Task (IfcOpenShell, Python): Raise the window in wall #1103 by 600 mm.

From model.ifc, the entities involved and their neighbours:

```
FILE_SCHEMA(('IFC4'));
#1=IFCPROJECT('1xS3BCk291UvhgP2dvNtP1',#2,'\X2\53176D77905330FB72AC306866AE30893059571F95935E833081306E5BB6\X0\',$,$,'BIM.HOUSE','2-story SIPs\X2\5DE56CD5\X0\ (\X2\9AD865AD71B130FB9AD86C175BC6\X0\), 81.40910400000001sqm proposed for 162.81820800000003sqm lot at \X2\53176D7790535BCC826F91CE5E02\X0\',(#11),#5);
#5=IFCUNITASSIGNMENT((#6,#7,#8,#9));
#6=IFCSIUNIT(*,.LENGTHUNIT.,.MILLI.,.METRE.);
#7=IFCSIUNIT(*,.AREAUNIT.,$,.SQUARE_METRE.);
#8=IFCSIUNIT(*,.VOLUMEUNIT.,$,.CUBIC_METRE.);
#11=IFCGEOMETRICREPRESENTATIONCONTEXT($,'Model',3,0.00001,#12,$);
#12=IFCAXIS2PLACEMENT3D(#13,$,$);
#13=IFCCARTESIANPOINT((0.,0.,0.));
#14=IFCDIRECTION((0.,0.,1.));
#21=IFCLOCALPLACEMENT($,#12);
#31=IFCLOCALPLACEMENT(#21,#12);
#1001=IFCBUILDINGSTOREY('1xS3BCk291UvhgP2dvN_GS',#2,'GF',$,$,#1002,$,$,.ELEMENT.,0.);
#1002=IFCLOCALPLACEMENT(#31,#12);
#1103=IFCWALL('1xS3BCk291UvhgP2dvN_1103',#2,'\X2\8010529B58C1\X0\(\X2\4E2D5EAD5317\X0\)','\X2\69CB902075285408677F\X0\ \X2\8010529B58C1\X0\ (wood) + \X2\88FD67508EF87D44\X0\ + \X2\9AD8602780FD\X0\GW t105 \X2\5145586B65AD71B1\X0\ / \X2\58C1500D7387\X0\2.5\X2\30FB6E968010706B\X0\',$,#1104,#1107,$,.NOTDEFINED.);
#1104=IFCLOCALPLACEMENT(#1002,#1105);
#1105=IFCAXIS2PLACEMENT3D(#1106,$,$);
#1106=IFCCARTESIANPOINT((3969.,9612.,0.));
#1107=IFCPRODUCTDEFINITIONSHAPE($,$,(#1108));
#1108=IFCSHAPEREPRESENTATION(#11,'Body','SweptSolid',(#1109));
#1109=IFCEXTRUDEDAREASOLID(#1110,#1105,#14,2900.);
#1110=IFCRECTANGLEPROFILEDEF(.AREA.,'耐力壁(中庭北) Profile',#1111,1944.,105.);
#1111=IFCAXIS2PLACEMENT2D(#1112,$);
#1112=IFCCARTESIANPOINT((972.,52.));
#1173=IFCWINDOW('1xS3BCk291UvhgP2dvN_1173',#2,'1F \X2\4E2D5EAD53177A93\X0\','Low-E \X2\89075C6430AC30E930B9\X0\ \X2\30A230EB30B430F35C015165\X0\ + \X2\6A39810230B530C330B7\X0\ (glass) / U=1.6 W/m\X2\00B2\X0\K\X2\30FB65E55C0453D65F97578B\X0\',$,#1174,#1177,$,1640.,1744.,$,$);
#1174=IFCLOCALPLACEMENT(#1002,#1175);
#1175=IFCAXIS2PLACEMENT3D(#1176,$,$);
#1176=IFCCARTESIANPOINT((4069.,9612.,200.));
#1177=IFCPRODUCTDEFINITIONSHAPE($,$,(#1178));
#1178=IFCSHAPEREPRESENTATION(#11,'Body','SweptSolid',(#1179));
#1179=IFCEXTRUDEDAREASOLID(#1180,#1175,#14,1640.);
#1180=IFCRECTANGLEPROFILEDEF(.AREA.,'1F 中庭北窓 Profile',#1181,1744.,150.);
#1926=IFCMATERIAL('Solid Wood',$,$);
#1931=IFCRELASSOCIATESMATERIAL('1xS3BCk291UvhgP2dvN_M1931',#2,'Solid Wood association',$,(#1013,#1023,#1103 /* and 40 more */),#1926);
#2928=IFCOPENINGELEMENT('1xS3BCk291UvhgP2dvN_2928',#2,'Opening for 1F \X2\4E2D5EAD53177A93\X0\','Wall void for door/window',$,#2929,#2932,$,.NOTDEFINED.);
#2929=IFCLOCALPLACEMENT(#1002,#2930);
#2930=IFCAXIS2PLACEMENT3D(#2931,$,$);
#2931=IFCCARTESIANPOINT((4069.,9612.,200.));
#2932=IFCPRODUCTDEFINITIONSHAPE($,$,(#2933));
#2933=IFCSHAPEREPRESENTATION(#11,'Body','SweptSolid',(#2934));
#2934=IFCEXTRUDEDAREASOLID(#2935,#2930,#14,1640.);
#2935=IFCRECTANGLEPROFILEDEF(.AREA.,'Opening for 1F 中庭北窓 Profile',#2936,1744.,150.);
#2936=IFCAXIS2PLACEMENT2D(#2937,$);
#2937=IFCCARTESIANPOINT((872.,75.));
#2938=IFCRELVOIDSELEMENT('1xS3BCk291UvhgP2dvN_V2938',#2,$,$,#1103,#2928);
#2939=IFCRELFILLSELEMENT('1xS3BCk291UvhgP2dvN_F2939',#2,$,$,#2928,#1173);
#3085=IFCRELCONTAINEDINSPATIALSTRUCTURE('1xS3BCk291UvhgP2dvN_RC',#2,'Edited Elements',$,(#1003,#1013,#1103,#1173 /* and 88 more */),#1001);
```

```python
import numpy as np
import ifcopenshell
import ifcopenshell.api.geometry
import ifcopenshell.util.placement
import ifcopenshell.util.unit

model = ifcopenshell.open("model.ifc")
unit_scale = ifcopenshell.util.unit.calculate_unit_scale(model)

window = model.by_guid("1xS3BCk291UvhgP2dvN_1173")
opening = window.FillsVoids[0].RelatingOpeningElement
dz = 600.0

shift = np.array([0.0, 0.0, dz])
# The window is not placed relative to its opening, so move both.
for product in (opening, window):
    matrix = ifcopenshell.util.placement.get_local_placement(product.ObjectPlacement)
    matrix[:3, 3] += shift
    ifcopenshell.api.geometry.edit_object_placement(model, product=product, matrix=matrix, is_si=False)

print(f"moved by {dz * unit_scale:+.3f} m")

model.write("model-out.ifc")
```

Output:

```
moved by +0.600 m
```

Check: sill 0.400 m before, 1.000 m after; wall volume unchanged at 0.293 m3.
